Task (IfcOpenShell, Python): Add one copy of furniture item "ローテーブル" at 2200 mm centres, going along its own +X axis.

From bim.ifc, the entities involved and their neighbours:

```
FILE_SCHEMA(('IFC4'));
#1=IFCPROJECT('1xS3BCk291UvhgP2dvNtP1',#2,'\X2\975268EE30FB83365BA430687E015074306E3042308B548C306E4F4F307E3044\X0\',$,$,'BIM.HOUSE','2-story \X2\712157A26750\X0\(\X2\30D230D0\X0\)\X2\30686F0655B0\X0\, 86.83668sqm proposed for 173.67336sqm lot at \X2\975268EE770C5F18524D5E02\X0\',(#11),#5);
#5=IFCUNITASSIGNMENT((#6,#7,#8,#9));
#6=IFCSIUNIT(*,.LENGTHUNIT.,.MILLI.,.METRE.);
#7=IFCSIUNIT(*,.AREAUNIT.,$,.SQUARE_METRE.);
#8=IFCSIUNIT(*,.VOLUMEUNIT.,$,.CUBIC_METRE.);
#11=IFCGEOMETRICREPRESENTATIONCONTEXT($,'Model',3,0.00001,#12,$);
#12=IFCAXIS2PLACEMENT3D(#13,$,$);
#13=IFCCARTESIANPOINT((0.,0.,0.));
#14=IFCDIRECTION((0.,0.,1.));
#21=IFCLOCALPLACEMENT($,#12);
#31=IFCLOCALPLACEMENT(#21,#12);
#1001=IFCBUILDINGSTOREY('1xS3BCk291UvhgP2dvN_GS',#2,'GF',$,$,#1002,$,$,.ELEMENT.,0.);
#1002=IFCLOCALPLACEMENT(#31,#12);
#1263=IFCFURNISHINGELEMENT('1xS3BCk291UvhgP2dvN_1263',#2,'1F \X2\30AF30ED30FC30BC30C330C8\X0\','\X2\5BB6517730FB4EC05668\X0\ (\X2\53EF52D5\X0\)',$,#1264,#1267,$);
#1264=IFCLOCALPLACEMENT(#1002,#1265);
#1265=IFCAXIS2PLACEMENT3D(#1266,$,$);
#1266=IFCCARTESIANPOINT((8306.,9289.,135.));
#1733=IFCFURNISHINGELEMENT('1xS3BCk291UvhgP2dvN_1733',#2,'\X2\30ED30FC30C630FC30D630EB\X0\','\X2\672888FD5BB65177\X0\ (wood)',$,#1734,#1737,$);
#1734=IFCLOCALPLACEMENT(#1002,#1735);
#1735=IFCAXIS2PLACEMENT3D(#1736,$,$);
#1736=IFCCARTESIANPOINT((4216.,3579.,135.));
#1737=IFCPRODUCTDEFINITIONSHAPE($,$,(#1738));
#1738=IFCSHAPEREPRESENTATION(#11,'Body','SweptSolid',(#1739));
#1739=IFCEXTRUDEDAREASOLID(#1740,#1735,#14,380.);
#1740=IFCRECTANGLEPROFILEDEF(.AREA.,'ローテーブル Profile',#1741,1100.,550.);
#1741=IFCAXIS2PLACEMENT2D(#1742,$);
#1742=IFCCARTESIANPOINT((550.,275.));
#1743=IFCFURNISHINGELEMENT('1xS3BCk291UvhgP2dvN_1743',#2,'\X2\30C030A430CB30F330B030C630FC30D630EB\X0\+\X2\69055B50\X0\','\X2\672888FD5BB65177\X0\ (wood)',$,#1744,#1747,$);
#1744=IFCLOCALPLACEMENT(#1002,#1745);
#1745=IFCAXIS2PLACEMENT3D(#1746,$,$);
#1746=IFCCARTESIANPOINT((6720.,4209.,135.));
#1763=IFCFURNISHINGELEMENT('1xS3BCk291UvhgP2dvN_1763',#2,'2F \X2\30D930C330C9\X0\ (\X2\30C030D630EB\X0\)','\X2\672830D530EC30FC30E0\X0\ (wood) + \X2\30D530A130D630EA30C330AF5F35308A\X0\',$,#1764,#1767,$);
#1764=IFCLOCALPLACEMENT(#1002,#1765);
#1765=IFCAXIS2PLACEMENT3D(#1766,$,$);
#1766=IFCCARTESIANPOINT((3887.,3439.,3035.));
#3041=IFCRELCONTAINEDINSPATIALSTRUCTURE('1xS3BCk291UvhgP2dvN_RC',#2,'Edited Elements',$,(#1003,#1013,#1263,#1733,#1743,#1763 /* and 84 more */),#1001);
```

```python
import ifcopenshell
import ifcopenshell.api.geometry
import ifcopenshell.api.root
import ifcopenshell.util.element
import ifcopenshell.util.placement
import ifcopenshell.util.unit

model = ifcopenshell.open("bim.ifc")
unit_scale = ifcopenshell.util.unit.calculate_unit_scale(model)


def reuse_history(source, copy):
    """copy_class also copies each property set's owner history, people and application; keep the originals."""
    for rel in copy.IsDefinedBy:
        if rel.is_a("IfcRelDefinesByProperties") and (history := rel.RelatingPropertyDefinition.OwnerHistory):
            rel.RelatingPropertyDefinition.OwnerHistory = source.OwnerHistory
            ifcopenshell.util.element.remove_deep2(model, history)


source = model.by_guid("1xS3BCk291UvhgP2dvN_1733")
base = ifcopenshell.util.placement.get_local_placement(source.ObjectPlacement)
step = base[:3, 0] * 2.2 / unit_scale

for i in range(1, 2):
    copy = ifcopenshell.api.root.copy_class(model, product=source)
    copy.Representation = ifcopenshell.util.element.copy_deep(
        model, source.Representation, exclude=["IfcGeometricRepresentationContext", "IfcRepresentationMap"]
    )
    reuse_history(source, copy)
    matrix = base.copy()
    matrix[:3, 3] += i * step
    print("added at", matrix[:3, 3].round(3) + 0.0)
    ifcopenshell.api.geometry.edit_object_placement(model, product=copy, matrix=matrix, is_si=False)

model.write("bim_v2.ifc")
```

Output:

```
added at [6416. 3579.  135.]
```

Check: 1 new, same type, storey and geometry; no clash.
